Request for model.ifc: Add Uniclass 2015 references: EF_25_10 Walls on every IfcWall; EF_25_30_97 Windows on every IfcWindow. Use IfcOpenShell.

First a look at what the model holds.

```python
import ifcopenshell

model = ifcopenshell.open("model.ifc")
print(model.schema)
print("classifications:", [c.Name for c in model.by_type("IfcClassification")])
for ifc_class in ("IfcDoor", "IfcRoof", "IfcStair", "IfcWall", "IfcWindow"):
    print(ifc_class, len(model.by_type(ifc_class)))
```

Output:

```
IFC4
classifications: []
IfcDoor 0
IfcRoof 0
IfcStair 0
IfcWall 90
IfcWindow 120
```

```python
import ifcopenshell
import ifcopenshell.api.classification

model = ifcopenshell.open("model.ifc")

system = ifcopenshell.api.classification.add_classification(model, classification="Uniclass 2015")

codes = {
    "IfcWall": ("EF_25_10", "Walls"),
    "IfcWindow": ("EF_25_30_97", "Windows"),
}
for ifc_class, (code, name) in codes.items():
    products = model.by_type(ifc_class)
    ifcopenshell.api.classification.add_reference(
        model, products=products, classification=system, identification=code, name=name
    )
    print(code, len(products))

model.write("model_edited.ifc")
```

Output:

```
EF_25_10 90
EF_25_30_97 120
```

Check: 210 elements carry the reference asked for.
